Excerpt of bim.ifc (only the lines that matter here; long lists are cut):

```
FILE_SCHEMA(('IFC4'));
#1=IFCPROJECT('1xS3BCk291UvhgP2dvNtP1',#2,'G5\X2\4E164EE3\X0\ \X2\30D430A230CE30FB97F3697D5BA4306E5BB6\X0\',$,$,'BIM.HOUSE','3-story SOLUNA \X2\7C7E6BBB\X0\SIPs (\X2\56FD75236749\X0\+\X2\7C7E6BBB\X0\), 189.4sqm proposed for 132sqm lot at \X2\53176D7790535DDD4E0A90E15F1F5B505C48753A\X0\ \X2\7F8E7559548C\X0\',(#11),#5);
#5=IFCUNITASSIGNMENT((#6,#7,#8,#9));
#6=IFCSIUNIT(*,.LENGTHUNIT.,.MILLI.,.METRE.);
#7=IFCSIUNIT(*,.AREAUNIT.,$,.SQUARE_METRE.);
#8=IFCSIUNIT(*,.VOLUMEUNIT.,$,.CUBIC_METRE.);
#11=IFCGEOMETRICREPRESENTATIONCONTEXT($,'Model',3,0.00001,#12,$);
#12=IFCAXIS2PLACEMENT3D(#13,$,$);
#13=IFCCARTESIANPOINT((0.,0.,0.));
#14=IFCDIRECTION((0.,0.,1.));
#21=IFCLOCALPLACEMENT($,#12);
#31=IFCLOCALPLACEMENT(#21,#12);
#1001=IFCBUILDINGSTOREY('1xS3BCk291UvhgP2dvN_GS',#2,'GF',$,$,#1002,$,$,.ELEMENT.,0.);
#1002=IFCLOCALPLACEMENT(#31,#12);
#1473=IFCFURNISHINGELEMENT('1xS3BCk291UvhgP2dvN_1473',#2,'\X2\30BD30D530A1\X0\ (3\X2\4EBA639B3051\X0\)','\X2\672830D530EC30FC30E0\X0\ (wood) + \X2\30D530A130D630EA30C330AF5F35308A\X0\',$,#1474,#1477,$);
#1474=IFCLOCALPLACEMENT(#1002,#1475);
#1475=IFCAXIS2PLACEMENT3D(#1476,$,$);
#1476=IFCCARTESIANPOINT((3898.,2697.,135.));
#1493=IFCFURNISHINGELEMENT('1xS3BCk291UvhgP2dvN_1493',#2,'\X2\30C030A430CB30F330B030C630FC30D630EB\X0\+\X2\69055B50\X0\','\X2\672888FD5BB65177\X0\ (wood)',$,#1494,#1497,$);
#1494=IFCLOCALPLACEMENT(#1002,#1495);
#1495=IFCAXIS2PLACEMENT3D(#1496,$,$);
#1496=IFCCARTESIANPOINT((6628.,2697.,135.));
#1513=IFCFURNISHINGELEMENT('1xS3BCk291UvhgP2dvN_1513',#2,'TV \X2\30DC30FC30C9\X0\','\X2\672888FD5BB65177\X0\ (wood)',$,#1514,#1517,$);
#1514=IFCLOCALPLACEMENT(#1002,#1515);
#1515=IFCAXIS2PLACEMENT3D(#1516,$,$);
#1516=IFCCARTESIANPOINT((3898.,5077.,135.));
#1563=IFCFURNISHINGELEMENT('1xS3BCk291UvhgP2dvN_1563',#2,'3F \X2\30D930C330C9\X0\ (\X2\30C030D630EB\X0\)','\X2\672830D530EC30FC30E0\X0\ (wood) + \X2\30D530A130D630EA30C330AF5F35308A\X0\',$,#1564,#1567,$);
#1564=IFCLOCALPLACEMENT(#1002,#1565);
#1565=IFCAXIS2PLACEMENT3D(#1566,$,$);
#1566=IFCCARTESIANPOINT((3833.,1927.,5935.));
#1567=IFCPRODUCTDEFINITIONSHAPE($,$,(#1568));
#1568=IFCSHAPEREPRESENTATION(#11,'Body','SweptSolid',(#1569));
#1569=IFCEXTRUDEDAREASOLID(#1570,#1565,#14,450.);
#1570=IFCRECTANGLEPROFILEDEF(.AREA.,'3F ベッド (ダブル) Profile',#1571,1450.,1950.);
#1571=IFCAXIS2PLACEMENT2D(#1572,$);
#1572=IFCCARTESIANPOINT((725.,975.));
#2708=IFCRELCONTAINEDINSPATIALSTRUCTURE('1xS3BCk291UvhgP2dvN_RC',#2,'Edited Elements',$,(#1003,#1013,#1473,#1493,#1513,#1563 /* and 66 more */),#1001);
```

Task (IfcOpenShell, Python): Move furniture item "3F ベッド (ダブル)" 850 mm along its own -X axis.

```python
import ifcopenshell
import ifcopenshell.api.geometry
import ifcopenshell.util.placement
import ifcopenshell.util.unit

model = ifcopenshell.open("bim.ifc")
unit_scale = ifcopenshell.util.unit.calculate_unit_scale(model)

item = model.by_guid("1xS3BCk291UvhgP2dvN_1563")
matrix = ifcopenshell.util.placement.get_local_placement(item.ObjectPlacement)
matrix[:3, 3] -= matrix[:3, 0] * 0.85 / unit_scale
ifcopenshell.api.geometry.edit_object_placement(model, product=item, matrix=matrix, is_si=False)

print(ifcopenshell.util.placement.get_local_placement(item.ObjectPlacement).round(3) + 0.0)

model.write("bim_rev.ifc")
```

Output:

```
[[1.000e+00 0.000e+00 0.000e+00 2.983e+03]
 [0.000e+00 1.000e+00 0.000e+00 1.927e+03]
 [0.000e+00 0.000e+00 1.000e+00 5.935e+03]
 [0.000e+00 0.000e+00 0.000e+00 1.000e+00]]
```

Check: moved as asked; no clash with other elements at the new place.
